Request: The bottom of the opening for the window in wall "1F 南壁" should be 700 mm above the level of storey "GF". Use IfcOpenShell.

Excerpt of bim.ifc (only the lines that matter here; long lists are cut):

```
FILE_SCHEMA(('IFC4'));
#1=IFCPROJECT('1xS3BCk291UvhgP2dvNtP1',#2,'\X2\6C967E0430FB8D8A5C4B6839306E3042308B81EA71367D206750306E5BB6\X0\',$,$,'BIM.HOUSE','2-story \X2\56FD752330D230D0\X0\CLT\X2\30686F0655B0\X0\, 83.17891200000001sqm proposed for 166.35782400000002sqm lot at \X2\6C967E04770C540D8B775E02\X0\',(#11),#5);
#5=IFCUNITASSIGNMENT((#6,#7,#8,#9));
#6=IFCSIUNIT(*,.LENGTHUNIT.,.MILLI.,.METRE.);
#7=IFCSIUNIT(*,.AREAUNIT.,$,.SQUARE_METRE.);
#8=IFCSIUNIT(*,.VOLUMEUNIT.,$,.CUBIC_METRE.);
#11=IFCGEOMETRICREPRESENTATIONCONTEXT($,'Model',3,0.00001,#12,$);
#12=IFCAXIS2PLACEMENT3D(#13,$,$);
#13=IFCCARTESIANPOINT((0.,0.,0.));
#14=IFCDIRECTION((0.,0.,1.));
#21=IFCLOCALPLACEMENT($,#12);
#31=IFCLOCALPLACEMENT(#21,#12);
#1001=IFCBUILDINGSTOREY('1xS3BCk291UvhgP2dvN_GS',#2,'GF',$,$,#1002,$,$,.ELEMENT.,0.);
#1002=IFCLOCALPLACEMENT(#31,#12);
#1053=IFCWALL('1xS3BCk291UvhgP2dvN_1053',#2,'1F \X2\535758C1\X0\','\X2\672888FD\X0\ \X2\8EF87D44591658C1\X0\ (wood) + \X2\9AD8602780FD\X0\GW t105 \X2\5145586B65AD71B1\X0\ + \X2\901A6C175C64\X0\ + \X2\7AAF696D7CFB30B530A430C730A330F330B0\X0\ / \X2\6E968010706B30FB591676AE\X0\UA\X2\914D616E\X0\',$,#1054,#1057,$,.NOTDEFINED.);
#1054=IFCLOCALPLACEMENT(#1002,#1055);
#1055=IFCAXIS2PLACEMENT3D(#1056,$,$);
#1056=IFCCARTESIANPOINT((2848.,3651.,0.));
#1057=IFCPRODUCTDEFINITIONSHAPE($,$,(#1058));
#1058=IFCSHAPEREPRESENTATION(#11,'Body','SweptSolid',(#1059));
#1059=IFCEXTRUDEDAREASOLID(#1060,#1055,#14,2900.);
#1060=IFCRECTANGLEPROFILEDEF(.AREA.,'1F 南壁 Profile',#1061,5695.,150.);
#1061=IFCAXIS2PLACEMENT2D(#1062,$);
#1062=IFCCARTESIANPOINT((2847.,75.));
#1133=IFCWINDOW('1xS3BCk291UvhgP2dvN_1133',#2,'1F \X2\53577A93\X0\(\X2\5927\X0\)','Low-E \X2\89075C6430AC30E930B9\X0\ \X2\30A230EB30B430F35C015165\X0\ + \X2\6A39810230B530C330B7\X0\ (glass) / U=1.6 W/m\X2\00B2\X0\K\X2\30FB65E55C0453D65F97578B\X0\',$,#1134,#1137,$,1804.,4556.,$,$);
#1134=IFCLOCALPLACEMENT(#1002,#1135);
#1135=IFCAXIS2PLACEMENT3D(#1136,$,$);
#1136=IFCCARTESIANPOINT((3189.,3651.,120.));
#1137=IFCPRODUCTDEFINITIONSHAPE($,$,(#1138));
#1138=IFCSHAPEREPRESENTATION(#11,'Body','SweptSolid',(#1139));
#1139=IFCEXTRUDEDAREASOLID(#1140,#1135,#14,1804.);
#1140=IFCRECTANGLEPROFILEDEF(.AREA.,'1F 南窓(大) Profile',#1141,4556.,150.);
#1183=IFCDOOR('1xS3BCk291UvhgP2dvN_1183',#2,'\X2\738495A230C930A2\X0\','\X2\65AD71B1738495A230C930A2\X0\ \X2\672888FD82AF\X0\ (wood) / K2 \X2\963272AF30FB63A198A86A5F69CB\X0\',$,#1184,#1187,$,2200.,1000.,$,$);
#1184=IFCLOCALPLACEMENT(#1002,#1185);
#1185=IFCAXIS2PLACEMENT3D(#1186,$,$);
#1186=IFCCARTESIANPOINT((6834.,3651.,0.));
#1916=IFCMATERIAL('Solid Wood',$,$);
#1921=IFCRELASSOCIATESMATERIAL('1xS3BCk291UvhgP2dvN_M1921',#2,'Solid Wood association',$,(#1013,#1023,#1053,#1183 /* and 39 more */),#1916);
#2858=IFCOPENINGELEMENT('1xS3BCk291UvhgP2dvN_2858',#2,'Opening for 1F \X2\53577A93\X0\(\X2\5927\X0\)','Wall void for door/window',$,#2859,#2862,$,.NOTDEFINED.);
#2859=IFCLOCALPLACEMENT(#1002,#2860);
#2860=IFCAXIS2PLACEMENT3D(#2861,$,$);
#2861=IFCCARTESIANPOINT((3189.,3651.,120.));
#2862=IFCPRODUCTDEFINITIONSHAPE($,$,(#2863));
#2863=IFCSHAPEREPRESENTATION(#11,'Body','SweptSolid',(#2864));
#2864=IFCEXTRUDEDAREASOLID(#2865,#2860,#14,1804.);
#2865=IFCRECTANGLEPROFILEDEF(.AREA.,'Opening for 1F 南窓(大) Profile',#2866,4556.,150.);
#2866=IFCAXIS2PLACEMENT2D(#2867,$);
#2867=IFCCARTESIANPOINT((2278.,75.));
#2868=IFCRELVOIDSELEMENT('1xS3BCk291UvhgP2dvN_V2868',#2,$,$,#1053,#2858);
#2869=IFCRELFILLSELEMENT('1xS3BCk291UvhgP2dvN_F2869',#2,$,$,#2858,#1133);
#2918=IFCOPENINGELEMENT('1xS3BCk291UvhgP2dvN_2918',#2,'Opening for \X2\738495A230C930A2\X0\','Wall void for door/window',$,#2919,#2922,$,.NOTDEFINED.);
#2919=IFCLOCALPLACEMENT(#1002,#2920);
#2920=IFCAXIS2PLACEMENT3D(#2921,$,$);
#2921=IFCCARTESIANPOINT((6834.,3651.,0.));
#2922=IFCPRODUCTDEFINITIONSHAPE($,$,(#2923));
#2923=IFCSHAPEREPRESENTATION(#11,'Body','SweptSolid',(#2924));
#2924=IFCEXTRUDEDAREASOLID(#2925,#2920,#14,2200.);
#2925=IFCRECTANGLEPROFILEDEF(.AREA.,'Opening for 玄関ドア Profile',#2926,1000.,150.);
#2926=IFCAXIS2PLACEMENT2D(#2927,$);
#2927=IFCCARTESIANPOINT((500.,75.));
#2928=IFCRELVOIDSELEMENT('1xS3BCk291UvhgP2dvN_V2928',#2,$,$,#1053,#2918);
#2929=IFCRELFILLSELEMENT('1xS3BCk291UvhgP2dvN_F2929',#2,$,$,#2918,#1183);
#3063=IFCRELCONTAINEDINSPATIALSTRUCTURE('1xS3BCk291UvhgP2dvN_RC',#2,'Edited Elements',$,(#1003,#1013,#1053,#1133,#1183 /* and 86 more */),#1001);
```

```python
import numpy as np
import ifcopenshell
import ifcopenshell.api.geometry
import ifcopenshell.geom
import ifcopenshell.util.element
import ifcopenshell.util.placement
import ifcopenshell.util.shape
import ifcopenshell.util.unit

model = ifcopenshell.open("bim.ifc")
unit_scale = ifcopenshell.util.unit.calculate_unit_scale(model)

window = model.by_guid("1xS3BCk291UvhgP2dvN_1133")
opening = window.FillsVoids[0].RelatingOpeningElement
storey = ifcopenshell.util.element.get_container(window, ifc_class="IfcBuildingStorey")
level = ifcopenshell.util.placement.get_local_placement(storey.ObjectPlacement)[2, 3]

# The opening's origin need not be at the sill, so measure its lowest point.
shape = ifcopenshell.geom.create_shape(ifcopenshell.geom.settings(), opening)
bottom = ifcopenshell.util.shape.get_shape_bottom_elevation(shape, shape.geometry) / unit_scale
dz = level + 0.7 / unit_scale - bottom

shift = np.array([0.0, 0.0, dz])
# The window is not placed relative to its opening, so move both.
for product in (opening, window):
    matrix = ifcopenshell.util.placement.get_local_placement(product.ObjectPlacement)
    matrix[:3, 3] += shift
    ifcopenshell.api.geometry.edit_object_placement(model, product=product, matrix=matrix, is_si=False)

print(f"moved by {dz * unit_scale:+.3f} m")

model.write("bim-out.ifc")
```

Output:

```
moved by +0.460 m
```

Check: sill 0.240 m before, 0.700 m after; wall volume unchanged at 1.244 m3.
